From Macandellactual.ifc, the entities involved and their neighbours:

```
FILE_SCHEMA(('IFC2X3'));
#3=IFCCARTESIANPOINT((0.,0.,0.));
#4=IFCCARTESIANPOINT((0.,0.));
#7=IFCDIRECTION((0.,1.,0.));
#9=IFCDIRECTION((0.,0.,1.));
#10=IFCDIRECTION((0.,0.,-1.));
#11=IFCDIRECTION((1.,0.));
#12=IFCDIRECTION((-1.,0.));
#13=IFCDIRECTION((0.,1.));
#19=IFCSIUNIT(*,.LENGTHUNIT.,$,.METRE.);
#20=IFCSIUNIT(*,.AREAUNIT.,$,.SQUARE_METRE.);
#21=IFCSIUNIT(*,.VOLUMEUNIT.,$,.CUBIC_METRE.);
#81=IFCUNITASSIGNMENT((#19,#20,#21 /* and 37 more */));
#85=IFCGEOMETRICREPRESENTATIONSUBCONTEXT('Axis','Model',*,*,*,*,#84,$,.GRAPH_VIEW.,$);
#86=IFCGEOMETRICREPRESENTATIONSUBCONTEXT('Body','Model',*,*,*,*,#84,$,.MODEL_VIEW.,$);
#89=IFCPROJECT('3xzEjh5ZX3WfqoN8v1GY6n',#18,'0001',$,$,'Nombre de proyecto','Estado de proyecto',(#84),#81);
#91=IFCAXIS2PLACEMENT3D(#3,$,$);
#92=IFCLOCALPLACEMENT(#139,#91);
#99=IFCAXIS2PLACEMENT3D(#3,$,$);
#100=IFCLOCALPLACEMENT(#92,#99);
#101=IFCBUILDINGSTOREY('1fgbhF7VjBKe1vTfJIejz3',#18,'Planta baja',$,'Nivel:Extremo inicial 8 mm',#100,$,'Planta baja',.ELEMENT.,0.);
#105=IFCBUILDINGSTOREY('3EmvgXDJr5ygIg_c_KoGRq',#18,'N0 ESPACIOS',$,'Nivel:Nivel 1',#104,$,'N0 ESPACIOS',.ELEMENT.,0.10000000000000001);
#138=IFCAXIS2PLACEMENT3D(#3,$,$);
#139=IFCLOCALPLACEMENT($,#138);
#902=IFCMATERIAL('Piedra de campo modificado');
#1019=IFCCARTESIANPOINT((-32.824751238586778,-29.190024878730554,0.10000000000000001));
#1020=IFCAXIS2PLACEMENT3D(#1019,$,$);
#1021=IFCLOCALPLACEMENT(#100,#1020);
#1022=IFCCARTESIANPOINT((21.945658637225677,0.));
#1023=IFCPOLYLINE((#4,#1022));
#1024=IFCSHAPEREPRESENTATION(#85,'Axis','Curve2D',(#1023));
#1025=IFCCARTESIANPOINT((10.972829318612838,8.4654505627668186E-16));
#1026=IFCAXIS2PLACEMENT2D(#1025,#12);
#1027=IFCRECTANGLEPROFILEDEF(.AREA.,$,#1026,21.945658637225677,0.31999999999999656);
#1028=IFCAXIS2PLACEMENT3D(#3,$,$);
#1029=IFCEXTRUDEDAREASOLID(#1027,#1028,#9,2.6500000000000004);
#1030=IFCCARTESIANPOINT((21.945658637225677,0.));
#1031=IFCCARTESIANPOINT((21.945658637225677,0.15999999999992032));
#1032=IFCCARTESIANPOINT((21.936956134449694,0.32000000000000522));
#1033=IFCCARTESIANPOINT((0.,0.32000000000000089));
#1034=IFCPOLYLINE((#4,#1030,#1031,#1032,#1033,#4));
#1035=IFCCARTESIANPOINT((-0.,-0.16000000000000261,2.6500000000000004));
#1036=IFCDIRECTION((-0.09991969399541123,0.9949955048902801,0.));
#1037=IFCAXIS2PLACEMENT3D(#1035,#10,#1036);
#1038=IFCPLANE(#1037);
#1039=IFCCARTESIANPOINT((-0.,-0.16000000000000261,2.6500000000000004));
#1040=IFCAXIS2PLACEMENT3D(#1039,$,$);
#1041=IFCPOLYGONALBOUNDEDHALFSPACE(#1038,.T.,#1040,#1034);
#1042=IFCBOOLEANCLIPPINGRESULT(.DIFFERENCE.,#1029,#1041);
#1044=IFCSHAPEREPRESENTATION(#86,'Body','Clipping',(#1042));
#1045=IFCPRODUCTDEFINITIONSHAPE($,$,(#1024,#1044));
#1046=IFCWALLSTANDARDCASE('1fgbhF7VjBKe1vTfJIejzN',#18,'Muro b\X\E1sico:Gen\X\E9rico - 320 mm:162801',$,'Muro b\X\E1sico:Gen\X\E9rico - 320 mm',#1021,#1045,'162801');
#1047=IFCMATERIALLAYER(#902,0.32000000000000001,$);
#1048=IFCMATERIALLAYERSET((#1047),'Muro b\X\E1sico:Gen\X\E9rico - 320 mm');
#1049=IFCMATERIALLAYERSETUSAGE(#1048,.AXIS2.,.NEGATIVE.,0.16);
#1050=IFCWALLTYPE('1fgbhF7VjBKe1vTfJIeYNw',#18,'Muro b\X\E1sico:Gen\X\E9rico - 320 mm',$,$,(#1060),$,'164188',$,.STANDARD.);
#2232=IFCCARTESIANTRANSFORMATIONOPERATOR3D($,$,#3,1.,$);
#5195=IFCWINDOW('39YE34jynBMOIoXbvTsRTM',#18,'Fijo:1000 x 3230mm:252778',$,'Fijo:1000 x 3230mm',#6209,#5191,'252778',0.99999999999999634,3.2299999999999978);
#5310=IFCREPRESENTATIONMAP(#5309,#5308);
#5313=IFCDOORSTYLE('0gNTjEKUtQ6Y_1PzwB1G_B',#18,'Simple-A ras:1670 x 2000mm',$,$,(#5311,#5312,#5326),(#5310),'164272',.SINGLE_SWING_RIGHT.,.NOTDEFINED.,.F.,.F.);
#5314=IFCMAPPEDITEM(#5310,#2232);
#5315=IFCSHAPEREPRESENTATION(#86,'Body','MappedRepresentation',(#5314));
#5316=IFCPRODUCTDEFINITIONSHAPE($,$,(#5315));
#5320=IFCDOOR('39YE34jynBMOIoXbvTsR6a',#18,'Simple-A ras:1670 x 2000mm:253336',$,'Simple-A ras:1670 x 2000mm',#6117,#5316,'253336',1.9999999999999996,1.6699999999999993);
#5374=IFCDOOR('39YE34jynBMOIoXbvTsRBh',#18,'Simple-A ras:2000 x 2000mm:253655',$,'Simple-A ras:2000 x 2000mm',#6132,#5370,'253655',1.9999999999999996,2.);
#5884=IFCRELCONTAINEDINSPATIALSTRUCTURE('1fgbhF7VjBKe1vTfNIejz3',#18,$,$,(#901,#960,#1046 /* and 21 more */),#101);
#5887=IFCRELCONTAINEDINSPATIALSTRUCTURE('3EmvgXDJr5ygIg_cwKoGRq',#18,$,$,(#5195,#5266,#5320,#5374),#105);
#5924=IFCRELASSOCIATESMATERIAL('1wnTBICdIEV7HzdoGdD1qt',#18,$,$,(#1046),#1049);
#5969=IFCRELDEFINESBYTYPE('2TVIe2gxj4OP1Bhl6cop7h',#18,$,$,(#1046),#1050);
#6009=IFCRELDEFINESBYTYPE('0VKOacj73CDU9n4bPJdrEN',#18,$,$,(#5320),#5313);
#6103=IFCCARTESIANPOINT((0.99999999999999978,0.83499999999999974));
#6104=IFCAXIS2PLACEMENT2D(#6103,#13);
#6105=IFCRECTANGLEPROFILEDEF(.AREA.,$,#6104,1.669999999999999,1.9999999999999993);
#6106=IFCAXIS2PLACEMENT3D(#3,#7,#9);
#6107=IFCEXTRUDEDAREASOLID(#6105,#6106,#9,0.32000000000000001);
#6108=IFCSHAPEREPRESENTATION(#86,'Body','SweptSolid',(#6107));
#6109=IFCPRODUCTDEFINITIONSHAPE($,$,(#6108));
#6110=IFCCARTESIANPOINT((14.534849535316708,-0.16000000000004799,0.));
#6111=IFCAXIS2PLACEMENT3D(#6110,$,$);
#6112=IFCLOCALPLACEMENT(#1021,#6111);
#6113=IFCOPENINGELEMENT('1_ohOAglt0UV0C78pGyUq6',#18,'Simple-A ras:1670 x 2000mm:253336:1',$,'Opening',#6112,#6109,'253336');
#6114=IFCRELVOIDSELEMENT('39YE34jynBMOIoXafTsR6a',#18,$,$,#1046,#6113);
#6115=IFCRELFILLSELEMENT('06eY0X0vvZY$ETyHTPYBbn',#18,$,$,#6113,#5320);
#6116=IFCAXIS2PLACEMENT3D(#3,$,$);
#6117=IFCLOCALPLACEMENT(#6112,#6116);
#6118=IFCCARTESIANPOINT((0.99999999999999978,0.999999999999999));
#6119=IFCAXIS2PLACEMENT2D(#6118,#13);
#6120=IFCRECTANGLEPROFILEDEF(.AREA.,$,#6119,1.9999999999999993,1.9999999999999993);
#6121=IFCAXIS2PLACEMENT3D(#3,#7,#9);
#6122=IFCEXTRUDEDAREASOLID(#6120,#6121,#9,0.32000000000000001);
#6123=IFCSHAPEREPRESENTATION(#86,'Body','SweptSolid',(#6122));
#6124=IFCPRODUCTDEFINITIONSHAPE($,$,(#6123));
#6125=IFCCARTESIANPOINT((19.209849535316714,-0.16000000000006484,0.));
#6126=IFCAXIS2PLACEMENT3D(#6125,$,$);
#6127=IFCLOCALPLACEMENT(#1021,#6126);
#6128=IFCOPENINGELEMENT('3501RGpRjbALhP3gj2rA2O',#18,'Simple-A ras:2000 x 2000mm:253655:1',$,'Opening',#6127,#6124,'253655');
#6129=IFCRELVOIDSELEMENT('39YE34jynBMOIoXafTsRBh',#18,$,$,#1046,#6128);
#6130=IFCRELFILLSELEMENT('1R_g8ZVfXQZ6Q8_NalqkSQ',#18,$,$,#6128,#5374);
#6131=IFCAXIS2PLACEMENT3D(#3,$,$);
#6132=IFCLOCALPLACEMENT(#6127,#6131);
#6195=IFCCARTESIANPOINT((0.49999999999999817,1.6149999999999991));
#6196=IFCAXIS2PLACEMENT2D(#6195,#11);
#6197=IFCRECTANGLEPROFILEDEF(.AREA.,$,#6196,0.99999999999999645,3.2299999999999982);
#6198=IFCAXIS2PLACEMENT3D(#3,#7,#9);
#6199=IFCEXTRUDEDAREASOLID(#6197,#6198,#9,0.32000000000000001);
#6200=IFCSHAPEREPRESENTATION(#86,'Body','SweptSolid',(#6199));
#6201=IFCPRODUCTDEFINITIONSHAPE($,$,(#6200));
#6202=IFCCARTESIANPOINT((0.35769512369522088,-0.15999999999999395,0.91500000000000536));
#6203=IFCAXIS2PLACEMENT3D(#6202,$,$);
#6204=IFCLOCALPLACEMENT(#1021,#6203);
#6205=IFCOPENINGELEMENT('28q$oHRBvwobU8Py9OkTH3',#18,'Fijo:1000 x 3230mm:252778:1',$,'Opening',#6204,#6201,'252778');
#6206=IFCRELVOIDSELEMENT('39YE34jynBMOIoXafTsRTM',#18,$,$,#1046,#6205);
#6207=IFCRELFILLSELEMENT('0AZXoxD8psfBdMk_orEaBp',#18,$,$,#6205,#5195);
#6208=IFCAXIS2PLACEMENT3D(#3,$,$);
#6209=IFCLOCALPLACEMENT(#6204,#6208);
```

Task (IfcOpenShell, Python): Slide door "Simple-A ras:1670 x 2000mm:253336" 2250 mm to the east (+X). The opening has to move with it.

```python
import ifcopenshell
import ifcopenshell.api.geometry
import ifcopenshell.util.placement
import ifcopenshell.util.unit

model = ifcopenshell.open("Macandellactual.ifc")
unit_scale = ifcopenshell.util.unit.calculate_unit_scale(model)

door = model.by_guid("39YE34jynBMOIoXbvTsR6a")
opening = door.FillsVoids[0].RelatingOpeningElement
wall = opening.VoidsElements[0].RelatingBuildingElement

wall_matrix = ifcopenshell.util.placement.get_local_placement(wall.ObjectPlacement)
shift = wall_matrix[:3, 0] * 2.25 / unit_scale
before = ifcopenshell.util.placement.get_local_placement(door.ObjectPlacement)[:3, 3].copy()

# The door is placed relative to its opening, so it follows when the opening moves.
matrix = ifcopenshell.util.placement.get_local_placement(opening.ObjectPlacement)
matrix[:3, 3] += shift
ifcopenshell.api.geometry.edit_object_placement(
    model, product=opening, matrix=matrix, is_si=False, should_transform_children=True
)

after = ifcopenshell.util.placement.get_local_placement(door.ObjectPlacement)[:3, 3]
print("door moved by", (after - before).round(3) + 0.0)

model.write("Macandellactual_rev.ifc")
```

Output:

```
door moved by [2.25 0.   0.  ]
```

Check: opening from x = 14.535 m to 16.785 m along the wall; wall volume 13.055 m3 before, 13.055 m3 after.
